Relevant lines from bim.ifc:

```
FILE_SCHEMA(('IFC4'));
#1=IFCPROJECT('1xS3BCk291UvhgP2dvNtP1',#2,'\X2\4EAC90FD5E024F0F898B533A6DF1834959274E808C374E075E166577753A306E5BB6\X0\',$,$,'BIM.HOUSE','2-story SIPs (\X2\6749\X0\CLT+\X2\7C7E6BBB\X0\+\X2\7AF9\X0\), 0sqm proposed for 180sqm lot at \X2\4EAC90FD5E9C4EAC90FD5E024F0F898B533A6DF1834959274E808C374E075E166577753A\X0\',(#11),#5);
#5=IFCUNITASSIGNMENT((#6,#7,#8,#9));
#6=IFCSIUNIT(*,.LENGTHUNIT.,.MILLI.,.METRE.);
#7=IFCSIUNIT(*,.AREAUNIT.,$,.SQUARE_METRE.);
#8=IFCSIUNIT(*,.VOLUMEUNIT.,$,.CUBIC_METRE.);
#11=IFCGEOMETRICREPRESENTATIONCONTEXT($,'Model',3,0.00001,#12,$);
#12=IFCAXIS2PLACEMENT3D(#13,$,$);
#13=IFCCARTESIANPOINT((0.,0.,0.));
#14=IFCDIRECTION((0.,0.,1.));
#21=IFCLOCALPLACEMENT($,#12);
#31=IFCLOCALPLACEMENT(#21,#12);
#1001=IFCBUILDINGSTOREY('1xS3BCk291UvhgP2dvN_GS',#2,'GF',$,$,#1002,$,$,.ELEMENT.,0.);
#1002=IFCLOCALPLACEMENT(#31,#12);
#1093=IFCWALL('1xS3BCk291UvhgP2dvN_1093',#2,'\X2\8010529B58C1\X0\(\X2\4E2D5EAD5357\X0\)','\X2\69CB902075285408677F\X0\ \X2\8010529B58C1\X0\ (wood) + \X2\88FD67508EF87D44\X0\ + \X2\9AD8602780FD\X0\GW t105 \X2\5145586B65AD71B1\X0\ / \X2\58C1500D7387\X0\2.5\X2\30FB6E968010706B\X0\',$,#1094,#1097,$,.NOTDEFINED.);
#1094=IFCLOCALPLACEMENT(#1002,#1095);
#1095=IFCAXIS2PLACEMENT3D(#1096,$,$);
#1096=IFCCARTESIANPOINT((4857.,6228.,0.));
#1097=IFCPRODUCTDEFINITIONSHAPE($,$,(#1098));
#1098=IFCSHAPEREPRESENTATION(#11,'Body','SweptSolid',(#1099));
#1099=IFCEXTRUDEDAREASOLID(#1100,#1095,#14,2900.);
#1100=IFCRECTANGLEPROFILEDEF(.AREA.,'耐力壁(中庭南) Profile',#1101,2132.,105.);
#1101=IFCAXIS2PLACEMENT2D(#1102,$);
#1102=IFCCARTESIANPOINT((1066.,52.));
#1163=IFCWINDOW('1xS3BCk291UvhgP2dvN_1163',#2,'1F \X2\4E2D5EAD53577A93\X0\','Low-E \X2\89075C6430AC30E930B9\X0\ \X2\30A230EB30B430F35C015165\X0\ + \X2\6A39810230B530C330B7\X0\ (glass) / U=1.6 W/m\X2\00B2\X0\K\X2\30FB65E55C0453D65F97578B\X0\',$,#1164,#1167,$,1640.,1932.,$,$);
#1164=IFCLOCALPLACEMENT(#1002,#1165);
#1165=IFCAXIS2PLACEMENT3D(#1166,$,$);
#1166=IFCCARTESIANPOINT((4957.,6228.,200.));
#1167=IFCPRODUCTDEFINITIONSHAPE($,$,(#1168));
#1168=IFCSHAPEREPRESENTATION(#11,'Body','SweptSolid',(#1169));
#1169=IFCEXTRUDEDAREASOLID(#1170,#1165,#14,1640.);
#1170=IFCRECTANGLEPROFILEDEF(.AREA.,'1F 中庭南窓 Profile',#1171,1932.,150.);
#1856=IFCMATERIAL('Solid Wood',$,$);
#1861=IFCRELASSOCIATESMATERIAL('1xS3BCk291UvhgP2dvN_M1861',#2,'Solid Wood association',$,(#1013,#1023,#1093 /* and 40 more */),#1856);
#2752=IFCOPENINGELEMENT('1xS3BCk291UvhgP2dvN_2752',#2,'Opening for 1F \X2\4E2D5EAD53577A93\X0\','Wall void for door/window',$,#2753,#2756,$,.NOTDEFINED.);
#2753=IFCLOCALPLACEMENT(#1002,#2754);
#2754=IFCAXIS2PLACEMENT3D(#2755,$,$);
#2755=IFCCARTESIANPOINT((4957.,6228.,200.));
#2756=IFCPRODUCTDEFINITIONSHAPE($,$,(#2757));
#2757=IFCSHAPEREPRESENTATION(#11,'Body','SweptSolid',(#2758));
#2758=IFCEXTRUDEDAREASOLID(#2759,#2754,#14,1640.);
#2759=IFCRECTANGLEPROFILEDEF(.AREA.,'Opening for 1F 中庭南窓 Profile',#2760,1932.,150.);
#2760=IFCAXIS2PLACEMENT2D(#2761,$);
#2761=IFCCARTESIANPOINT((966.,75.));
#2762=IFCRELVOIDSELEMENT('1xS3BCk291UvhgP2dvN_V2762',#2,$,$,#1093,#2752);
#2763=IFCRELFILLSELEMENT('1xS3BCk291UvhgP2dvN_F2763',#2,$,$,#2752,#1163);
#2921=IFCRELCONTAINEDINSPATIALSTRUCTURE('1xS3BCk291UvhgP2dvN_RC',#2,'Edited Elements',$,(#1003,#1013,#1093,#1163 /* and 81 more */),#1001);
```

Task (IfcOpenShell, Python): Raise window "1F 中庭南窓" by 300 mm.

```python
import numpy as np
import ifcopenshell
import ifcopenshell.api.geometry
import ifcopenshell.util.placement
import ifcopenshell.util.unit

model = ifcopenshell.open("bim.ifc")
unit_scale = ifcopenshell.util.unit.calculate_unit_scale(model)

window = model.by_id(1163)
opening = window.FillsVoids[0].RelatingOpeningElement
dz = 300.0

shift = np.array([0.0, 0.0, dz])
# The window is not placed relative to its opening, so move both.
for product in (opening, window):
    matrix = ifcopenshell.util.placement.get_local_placement(product.ObjectPlacement)
    matrix[:3, 3] += shift
    ifcopenshell.api.geometry.edit_object_placement(model, product=product, matrix=matrix, is_si=False)

print(f"moved by {dz * unit_scale:+.3f} m")

model.write("bim_edited.ifc")
```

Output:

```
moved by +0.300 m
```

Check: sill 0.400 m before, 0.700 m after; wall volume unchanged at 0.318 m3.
